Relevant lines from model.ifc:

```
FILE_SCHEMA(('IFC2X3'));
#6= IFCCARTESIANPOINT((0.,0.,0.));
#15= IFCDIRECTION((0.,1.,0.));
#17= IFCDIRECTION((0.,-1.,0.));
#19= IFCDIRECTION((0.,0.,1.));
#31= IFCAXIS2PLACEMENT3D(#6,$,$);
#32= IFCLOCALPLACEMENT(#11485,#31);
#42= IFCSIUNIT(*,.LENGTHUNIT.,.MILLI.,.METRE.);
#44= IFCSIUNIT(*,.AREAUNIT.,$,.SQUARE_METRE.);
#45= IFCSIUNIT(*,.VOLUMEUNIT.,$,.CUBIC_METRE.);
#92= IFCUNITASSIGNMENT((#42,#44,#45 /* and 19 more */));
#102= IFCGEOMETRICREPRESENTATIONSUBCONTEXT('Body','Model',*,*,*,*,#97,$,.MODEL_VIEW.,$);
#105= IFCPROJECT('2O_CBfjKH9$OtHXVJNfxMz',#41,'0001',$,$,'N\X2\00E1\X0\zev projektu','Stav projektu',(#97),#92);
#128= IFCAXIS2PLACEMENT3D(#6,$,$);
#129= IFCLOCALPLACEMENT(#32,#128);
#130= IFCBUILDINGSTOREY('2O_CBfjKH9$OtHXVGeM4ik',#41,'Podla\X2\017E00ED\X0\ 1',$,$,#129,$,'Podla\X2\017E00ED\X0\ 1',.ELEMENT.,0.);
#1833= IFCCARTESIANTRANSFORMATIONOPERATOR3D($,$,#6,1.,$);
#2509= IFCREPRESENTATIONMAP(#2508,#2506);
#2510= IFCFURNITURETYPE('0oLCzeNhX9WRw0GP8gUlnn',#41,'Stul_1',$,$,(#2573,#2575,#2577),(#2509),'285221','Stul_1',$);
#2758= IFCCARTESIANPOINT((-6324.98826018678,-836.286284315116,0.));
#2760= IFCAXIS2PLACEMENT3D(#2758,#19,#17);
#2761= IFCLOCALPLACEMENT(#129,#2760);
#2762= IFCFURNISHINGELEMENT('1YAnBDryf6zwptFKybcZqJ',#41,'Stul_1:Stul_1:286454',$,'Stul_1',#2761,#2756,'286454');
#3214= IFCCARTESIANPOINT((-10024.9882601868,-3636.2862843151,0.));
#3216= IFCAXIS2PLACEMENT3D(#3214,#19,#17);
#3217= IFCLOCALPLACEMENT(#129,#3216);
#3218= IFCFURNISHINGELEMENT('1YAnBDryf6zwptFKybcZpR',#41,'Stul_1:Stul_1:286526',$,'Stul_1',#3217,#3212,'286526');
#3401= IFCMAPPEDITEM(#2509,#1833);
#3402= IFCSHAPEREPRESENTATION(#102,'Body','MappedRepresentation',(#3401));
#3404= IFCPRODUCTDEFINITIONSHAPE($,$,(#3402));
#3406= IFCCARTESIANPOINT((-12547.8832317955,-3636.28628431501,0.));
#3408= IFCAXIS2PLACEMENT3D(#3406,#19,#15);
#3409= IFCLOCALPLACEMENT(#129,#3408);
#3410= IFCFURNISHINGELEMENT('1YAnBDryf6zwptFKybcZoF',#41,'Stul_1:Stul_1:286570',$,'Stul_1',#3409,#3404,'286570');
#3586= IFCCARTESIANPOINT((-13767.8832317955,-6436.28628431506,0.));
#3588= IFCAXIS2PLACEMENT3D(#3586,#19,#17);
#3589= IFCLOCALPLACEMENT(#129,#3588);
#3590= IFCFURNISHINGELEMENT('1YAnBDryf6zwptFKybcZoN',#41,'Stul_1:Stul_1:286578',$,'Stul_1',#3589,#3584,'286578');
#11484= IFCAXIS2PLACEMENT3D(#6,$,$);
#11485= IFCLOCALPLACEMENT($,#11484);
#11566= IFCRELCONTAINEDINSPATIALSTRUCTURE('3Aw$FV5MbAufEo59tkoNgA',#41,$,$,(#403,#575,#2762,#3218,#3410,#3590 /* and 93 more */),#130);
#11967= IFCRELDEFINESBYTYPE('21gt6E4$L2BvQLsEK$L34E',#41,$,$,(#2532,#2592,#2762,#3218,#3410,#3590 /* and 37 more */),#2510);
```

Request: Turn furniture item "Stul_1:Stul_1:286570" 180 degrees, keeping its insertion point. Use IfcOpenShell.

```python
import ifcopenshell
import ifcopenshell.api.geometry
import ifcopenshell.util.placement

model = ifcopenshell.open("model.ifc")

item = model.by_guid("1YAnBDryf6zwptFKybcZoF")
matrix = ifcopenshell.util.placement.get_local_placement(item.ObjectPlacement)
matrix = matrix @ ifcopenshell.util.placement.rotation(180, "Z")
ifcopenshell.api.geometry.edit_object_placement(model, product=item, matrix=matrix, is_si=False)

print(ifcopenshell.util.placement.get_local_placement(item.ObjectPlacement).round(3) + 0.0)

model.write("model-out.ifc")
```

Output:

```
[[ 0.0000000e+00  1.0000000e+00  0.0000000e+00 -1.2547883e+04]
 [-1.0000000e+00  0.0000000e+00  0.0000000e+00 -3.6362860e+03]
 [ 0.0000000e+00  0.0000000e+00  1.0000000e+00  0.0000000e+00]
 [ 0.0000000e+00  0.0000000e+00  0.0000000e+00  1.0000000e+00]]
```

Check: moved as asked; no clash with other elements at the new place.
